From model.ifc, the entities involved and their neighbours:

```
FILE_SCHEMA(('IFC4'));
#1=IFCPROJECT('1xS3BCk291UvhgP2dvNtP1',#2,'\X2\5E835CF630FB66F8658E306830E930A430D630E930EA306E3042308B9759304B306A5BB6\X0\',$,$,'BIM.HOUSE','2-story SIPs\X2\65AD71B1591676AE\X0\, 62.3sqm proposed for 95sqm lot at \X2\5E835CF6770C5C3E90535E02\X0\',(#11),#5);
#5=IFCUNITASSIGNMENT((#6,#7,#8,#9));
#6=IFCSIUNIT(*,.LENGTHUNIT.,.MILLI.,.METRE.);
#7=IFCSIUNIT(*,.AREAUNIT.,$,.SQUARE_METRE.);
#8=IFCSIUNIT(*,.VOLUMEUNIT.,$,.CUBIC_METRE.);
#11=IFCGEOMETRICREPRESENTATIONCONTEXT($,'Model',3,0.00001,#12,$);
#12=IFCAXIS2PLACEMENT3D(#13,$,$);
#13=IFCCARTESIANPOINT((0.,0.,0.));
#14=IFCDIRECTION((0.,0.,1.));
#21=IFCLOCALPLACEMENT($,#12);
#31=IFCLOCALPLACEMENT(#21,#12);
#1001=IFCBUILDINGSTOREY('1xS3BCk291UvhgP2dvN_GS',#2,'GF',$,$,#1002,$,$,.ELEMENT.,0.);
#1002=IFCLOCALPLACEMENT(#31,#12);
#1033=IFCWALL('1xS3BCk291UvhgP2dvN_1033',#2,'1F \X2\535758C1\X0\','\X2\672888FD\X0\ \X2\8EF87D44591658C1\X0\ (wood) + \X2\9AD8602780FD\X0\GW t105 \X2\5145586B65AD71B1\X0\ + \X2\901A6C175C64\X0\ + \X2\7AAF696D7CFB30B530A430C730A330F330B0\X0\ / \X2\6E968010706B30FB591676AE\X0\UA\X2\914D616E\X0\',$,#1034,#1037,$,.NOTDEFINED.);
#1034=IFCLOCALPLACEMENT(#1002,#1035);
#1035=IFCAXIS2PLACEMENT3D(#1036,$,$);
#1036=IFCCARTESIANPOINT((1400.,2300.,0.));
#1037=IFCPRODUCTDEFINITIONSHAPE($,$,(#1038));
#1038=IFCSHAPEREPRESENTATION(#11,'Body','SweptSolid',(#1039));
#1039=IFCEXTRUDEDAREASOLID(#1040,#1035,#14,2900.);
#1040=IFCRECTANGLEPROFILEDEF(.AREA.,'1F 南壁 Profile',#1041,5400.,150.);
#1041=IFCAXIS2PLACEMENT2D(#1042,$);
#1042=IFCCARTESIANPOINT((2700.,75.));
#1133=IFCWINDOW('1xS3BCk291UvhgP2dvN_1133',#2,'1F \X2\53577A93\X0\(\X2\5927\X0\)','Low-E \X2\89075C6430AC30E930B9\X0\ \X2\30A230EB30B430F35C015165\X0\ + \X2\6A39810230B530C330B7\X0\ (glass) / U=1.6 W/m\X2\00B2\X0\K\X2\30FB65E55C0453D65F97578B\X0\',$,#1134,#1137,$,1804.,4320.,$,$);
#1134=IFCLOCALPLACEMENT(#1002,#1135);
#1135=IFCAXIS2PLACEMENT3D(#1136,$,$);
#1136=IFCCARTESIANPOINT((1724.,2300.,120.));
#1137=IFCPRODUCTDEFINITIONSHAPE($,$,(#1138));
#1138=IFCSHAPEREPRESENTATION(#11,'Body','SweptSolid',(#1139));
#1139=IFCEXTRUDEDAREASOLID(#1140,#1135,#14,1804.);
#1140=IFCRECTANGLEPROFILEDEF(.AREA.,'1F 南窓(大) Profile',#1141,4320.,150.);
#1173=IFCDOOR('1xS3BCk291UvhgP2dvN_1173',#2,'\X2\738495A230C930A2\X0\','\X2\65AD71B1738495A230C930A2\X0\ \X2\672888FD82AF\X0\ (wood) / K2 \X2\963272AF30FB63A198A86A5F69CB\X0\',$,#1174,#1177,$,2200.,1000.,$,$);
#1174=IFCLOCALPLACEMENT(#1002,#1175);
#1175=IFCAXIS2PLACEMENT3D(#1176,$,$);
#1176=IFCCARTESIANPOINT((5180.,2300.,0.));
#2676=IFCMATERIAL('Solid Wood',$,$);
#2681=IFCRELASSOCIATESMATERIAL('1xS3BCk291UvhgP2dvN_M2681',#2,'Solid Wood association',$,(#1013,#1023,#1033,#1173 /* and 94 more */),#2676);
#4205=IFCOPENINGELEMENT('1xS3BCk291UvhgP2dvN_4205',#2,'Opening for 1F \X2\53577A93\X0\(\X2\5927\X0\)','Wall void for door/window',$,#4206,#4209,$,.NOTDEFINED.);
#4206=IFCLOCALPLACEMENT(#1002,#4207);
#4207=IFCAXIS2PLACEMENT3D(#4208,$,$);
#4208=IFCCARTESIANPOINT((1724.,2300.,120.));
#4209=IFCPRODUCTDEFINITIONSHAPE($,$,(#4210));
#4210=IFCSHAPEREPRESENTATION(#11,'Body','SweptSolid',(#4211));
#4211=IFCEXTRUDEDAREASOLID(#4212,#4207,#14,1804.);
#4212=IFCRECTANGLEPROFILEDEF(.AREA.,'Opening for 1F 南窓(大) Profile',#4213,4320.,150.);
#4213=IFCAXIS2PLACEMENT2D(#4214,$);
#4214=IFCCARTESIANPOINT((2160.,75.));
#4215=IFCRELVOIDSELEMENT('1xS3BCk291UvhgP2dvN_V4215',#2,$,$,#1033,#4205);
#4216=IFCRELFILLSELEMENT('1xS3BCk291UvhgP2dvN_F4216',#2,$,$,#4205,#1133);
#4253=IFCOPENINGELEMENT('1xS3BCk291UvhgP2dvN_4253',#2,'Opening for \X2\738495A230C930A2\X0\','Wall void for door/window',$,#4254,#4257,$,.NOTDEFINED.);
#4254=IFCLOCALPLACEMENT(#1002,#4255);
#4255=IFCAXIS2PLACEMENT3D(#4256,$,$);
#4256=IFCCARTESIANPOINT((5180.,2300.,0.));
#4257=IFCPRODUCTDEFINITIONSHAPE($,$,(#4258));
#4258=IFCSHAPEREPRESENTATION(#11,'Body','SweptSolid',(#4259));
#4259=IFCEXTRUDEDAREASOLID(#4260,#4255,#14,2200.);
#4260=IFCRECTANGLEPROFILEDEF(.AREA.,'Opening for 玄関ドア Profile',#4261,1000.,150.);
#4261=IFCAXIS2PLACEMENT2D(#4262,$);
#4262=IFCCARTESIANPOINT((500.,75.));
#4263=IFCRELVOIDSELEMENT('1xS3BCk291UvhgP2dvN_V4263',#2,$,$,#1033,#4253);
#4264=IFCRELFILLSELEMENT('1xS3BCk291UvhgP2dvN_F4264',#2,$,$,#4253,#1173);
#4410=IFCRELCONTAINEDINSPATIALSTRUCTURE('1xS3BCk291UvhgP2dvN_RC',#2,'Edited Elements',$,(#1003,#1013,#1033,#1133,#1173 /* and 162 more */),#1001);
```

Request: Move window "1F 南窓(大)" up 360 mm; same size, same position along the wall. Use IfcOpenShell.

```python
import numpy as np
import ifcopenshell
import ifcopenshell.api.geometry
import ifcopenshell.util.placement
import ifcopenshell.util.unit

model = ifcopenshell.open("model.ifc")
unit_scale = ifcopenshell.util.unit.calculate_unit_scale(model)

window = model.by_guid("1xS3BCk291UvhgP2dvN_1133")
opening = window.FillsVoids[0].RelatingOpeningElement
dz = 0.36 / unit_scale

shift = np.array([0.0, 0.0, dz])
# The window is not placed relative to its opening, so move both.
for product in (opening, window):
    matrix = ifcopenshell.util.placement.get_local_placement(product.ObjectPlacement)
    matrix[:3, 3] += shift
    ifcopenshell.api.geometry.edit_object_placement(model, product=product, matrix=matrix, is_si=False)

print(f"moved by {dz * unit_scale:+.3f} m")

model.write("model-out.ifc")
```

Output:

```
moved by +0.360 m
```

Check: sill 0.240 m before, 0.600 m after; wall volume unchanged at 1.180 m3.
